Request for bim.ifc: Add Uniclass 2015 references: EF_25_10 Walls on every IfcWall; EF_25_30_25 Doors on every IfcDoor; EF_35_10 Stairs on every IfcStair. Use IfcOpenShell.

First a look at what the model holds.

```python
import ifcopenshell

model = ifcopenshell.open("bim.ifc")
print(model.schema)
print("classifications:", [c.Name for c in model.by_type("IfcClassification")])
for ifc_class in ("IfcDoor", "IfcRoof", "IfcStair", "IfcWall", "IfcWindow"):
    print(ifc_class, len(model.by_type(ifc_class)))
```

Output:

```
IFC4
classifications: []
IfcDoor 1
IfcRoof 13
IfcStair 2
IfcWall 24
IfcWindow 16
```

```python
import ifcopenshell
import ifcopenshell.api.classification

model = ifcopenshell.open("bim.ifc")

system = ifcopenshell.api.classification.add_classification(model, classification="Uniclass 2015")

codes = {
    "IfcWall": ("EF_25_10", "Walls"),
    "IfcDoor": ("EF_25_30_25", "Doors"),
    "IfcStair": ("EF_35_10", "Stairs"),
}
for ifc_class, (code, name) in codes.items():
    products = model.by_type(ifc_class)
    ifcopenshell.api.classification.add_reference(
        model, products=products, classification=system, identification=code, name=name
    )
    print(code, len(products))

model.write("bim_v2.ifc")
```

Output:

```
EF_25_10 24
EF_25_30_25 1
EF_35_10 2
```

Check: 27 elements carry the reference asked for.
